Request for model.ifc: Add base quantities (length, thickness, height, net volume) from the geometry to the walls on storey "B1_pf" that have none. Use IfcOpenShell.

First a look at what the model holds.

```python
import ifcopenshell
import ifcopenshell.util.element
import ifcopenshell.util.unit

model = ifcopenshell.open("model.ifc")
print(model.schema)
for unit_type in ("LENGTHUNIT", "AREAUNIT", "VOLUMEUNIT"):
    print(unit_type, ifcopenshell.util.unit.calculate_unit_scale(model, unit_type))
storey = next(s for s in model.by_type("IfcBuildingStorey") if s.Name == "B1_pf")
walls = [e for e in ifcopenshell.util.element.get_decomposition(storey) if e.is_a("IfcWall")]
for e in sorted(walls, key=lambda e: e.id()):
    print(e.id(), e.is_a(), e.Name, list(ifcopenshell.util.element.get_psets(e, qtos_only=True)), sep=" | ")
```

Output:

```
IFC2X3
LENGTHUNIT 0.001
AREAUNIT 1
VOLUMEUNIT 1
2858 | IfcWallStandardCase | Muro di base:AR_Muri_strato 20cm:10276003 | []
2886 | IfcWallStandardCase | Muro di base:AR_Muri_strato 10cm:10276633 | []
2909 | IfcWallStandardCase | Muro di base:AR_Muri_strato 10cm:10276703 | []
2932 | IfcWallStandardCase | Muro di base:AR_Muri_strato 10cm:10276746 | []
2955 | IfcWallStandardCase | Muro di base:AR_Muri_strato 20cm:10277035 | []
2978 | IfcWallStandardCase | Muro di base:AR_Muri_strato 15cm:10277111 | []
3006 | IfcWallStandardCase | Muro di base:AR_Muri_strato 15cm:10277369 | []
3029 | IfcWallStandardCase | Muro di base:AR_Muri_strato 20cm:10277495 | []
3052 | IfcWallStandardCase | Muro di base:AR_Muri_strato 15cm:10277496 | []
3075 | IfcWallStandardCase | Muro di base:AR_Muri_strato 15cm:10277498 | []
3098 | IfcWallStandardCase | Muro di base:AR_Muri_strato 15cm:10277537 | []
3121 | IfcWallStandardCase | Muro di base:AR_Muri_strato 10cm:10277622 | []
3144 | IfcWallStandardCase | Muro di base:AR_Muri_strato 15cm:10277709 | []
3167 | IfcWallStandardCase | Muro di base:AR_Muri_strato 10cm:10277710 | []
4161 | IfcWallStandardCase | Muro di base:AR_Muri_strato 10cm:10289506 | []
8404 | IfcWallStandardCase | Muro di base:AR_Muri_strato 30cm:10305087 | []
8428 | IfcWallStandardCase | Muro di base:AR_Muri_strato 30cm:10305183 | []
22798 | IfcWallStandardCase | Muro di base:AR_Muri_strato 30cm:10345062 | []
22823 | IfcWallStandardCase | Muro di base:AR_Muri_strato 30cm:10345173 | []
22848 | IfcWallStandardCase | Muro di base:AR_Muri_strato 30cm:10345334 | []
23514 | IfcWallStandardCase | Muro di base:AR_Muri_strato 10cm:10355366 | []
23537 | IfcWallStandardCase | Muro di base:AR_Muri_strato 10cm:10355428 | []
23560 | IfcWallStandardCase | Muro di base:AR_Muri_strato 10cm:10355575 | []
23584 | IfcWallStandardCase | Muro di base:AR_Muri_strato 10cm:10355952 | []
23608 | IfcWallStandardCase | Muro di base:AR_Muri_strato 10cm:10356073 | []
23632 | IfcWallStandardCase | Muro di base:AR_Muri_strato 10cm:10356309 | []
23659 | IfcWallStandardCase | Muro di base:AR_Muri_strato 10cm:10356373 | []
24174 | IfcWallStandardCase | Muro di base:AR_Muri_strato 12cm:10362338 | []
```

```python
import ifcopenshell
import ifcopenshell.api.pset
import ifcopenshell.geom
import ifcopenshell.util.element
import ifcopenshell.util.shape
import ifcopenshell.util.unit

model = ifcopenshell.open("model.ifc")
unit_scale = ifcopenshell.util.unit.calculate_unit_scale(model)
volume_scale = ifcopenshell.util.unit.calculate_unit_scale(model, "VOLUMEUNIT")
settings = ifcopenshell.geom.settings()

storey = next(s for s in model.by_type("IfcBuildingStorey") if s.Name == "B1_pf")
walls = [e for e in ifcopenshell.util.element.get_decomposition(storey) if e.is_a("IfcWall")]

for e in sorted(walls, key=lambda e: e.id()):
    if ifcopenshell.util.element.get_psets(e, qtos_only=True, should_inherit=False):
        continue
    # Geometry comes back in metres, in the element's own axes.
    shape = ifcopenshell.geom.create_shape(settings, e)
    values = {
        "Length": ifcopenshell.util.shape.get_x(shape.geometry) / unit_scale,
        "Width": ifcopenshell.util.shape.get_y(shape.geometry) / unit_scale,
        "Height": ifcopenshell.util.shape.get_z(shape.geometry) / unit_scale,
        "NetVolume": ifcopenshell.util.shape.get_volume(shape.geometry) / volume_scale,
    }
    qto = ifcopenshell.api.pset.add_qto(model, product=e, name="BaseQuantities")
    ifcopenshell.api.pset.edit_qto(model, qto=qto, properties=values)
    print(e.id(), {k: round(v, 3) for k, v in values.items()})

model.write("model-out.ifc")
```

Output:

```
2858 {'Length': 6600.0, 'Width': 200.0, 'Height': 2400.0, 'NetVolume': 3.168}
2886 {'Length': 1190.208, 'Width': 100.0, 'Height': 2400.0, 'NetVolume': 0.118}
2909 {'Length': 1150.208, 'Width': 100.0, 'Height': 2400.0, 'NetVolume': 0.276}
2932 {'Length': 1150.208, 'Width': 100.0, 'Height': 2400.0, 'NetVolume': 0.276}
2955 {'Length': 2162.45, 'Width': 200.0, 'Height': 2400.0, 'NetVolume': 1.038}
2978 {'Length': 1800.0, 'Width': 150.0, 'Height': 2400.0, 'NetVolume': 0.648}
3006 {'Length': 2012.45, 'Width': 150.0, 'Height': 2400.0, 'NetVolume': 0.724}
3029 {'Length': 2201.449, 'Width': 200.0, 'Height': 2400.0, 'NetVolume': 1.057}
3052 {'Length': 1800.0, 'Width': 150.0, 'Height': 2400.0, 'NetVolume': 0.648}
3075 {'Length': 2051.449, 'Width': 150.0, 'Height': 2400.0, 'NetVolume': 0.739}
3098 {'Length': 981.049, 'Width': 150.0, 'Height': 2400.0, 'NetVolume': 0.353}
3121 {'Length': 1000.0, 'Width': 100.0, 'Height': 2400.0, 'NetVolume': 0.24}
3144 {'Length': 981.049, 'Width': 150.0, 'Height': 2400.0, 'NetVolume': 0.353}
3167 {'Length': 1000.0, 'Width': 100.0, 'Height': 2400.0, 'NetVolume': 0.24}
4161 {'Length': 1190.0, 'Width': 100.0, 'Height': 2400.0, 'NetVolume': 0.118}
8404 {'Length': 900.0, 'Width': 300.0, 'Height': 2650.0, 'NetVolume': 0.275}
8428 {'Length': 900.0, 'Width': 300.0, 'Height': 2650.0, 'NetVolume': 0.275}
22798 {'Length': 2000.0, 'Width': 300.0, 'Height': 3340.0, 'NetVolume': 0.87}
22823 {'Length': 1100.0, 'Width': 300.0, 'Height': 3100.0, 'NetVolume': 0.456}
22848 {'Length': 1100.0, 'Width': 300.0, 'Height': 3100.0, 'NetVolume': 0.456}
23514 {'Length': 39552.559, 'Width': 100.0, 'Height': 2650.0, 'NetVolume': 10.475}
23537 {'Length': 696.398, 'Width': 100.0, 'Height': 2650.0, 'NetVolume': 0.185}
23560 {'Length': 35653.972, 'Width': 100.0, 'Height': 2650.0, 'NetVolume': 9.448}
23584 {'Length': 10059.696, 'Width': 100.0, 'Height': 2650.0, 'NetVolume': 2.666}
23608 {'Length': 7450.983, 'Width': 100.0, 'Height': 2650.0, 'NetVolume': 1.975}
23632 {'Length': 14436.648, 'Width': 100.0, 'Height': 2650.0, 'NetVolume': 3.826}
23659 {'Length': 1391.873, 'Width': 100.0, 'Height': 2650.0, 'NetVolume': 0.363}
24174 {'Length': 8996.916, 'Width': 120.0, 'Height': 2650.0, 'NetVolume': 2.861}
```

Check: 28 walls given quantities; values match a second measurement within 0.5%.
